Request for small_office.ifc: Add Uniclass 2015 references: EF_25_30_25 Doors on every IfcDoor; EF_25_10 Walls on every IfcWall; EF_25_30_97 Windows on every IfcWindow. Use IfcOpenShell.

First a look at what the model holds.

```python
import ifcopenshell

model = ifcopenshell.open("small_office.ifc")
print(model.schema)
print("classifications:", [c.Name for c in model.by_type("IfcClassification")])
for ifc_class in ("IfcDoor", "IfcRoof", "IfcStair", "IfcWall", "IfcWindow"):
    print(ifc_class, len(model.by_type(ifc_class)))
```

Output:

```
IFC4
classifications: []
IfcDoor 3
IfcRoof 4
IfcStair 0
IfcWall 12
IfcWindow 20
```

```python
import ifcopenshell
import ifcopenshell.api.classification

model = ifcopenshell.open("small_office.ifc")

system = ifcopenshell.api.classification.add_classification(model, classification="Uniclass 2015")

codes = {
    "IfcDoor": ("EF_25_30_25", "Doors"),
    "IfcWall": ("EF_25_10", "Walls"),
    "IfcWindow": ("EF_25_30_97", "Windows"),
}
for ifc_class, (code, name) in codes.items():
    products = model.by_type(ifc_class)
    ifcopenshell.api.classification.add_reference(
        model, products=products, classification=system, identification=code, name=name
    )
    print(code, len(products))

model.write("small_office_edited.ifc")
```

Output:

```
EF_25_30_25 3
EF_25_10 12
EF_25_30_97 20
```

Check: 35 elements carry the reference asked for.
